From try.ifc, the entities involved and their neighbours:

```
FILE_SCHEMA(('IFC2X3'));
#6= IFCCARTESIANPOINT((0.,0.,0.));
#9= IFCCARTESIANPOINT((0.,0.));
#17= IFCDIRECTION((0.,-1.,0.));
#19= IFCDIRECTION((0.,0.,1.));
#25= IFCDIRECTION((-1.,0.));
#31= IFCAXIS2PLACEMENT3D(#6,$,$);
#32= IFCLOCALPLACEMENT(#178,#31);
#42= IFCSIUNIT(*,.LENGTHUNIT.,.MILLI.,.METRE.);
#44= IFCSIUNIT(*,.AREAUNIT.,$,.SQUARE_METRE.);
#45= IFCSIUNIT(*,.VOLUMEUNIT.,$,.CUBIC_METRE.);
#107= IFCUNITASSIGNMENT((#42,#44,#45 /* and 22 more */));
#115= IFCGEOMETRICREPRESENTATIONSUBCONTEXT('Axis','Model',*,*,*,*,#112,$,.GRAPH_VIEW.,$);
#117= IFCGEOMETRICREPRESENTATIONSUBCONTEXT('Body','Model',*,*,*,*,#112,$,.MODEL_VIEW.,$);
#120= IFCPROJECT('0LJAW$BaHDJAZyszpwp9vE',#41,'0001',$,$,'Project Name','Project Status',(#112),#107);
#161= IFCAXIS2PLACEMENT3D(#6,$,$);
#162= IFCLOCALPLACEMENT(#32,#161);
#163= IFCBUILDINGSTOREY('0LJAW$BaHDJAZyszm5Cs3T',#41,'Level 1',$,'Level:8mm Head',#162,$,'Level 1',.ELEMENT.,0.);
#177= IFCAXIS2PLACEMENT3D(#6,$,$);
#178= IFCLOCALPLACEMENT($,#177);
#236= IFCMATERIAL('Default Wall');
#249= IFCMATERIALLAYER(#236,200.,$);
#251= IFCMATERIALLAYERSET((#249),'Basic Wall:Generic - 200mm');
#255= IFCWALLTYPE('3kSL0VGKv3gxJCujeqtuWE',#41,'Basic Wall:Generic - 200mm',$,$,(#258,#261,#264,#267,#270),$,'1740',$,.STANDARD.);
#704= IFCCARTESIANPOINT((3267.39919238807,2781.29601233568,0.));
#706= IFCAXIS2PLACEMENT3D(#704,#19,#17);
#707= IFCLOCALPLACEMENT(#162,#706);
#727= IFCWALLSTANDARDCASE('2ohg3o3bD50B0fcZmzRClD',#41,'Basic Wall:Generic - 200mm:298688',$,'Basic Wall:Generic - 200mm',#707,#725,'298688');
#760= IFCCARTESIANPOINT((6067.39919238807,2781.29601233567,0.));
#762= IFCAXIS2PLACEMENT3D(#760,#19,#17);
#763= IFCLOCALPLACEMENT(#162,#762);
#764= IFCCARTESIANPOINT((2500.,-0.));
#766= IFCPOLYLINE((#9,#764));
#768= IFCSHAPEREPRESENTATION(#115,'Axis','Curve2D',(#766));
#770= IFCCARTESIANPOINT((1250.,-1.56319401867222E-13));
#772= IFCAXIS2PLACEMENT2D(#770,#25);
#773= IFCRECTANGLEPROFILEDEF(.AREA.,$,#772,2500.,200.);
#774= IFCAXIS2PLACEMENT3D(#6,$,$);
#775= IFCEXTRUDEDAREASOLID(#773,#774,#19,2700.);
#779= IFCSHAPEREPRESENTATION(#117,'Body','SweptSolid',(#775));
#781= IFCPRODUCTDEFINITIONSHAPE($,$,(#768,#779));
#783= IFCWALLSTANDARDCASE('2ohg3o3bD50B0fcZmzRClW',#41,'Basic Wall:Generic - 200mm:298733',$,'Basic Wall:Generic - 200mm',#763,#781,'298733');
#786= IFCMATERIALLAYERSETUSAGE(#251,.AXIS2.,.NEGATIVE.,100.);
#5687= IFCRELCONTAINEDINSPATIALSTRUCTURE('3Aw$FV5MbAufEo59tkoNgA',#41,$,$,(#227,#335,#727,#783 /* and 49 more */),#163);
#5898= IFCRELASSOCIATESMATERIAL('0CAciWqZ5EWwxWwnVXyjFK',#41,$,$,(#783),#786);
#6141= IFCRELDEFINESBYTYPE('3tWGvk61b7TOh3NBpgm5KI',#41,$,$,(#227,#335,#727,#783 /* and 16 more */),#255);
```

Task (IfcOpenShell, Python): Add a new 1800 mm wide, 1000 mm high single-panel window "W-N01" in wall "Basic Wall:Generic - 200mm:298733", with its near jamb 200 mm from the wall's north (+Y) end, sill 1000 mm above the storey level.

```python
import numpy as np
import ifcopenshell
import ifcopenshell.api.feature
import ifcopenshell.api.geometry
import ifcopenshell.api.root
import ifcopenshell.api.spatial
import ifcopenshell.api.type
import ifcopenshell.geom
import ifcopenshell.util.element
import ifcopenshell.util.placement
import ifcopenshell.util.representation
import ifcopenshell.util.shape
import ifcopenshell.util.unit

model = ifcopenshell.open("try.ifc")
unit_scale = ifcopenshell.util.unit.calculate_unit_scale(model)
settings = ifcopenshell.geom.settings()


def volume(element):
    """Net volume in cubic metres, openings subtracted."""
    shape = ifcopenshell.geom.create_shape(settings, element)
    return ifcopenshell.util.shape.get_volume(shape.geometry)


wall = model.by_id(783)
storey = ifcopenshell.util.element.get_container(wall, ifc_class="IfcBuildingStorey")
context = ifcopenshell.util.representation.get_context(model, "Model", "Body", "MODEL_VIEW")
before = volume(wall)

width, height, from_end, sill = 1.8, 1, 0.2, 1  # metres

# The wall runs along its own X axis, and the end named is its -X end.
wall_shape = ifcopenshell.geom.create_shape(settings, wall)
x, y, z = ifcopenshell.util.shape.get_vertices(wall_shape.geometry).T
start = x.min() + from_end
face, thickness = float(y.min()), float(y.max() - y.min())
wall_matrix = ifcopenshell.util.placement.get_local_placement(wall.ObjectPlacement)
level = ifcopenshell.util.placement.get_local_placement(storey.ObjectPlacement)[2, 3]


def in_wall(x, y):
    """Placement at x, y metres in the wall's axes, at sill height."""
    matrix = wall_matrix.copy()
    matrix[:, 3] = wall_matrix @ np.array([x / unit_scale, y / unit_scale, 0.0, 1.0])
    matrix[2, 3] = level + sill / unit_scale
    return matrix


# Opening: a box that overshoots both wall faces by 50 mm.
opening = ifcopenshell.api.root.create_entity(model, ifc_class="IfcOpeningElement")
box = ifcopenshell.api.geometry.add_wall_representation(
    model, context=context, length=width, height=height, thickness=thickness + 0.1
)
ifcopenshell.api.geometry.assign_representation(model, product=opening, representation=box)
ifcopenshell.api.geometry.edit_object_placement(model, product=opening, matrix=in_wall(start, face - 0.05), is_si=False)
ifcopenshell.api.feature.add_feature(model, feature=opening, element=wall)

window = ifcopenshell.api.root.create_entity(model, ifc_class="IfcWindow", name="W-N01")
window.OverallWidth, window.OverallHeight = width / unit_scale, height / unit_scale
body = ifcopenshell.api.geometry.add_window_representation(
    model,
    context=context,
    overall_width=window.OverallWidth,
    overall_height=window.OverallHeight,
    partition_type="SINGLE_PANEL",
)
ifcopenshell.api.geometry.assign_representation(model, product=window, representation=body)
ifcopenshell.api.spatial.assign_container(model, products=[window], relating_structure=storey)
fills = ifcopenshell.api.feature.add_filling(model, opening=opening, element=window)
fills.OwnerHistory = window.OwnerHistory  # required in IFC2X3

# IFC2X3 keeps the operation on the window style.
style = ifcopenshell.api.root.create_entity(model, ifc_class="IfcWindowStyle", name="W-N01")
style.OperationType, style.ConstructionType = "SINGLE_PANEL", "NOTDEFINED"
style.ParameterTakesPrecedence = style.Sizeable = False
ifcopenshell.api.type.assign_type(model, related_objects=[window], relating_type=style)

# Centre the window in the wall's thickness.
ifcopenshell.api.geometry.edit_object_placement(model, product=window, matrix=in_wall(start, face), is_si=False)
window_shape = ifcopenshell.geom.create_shape(settings, window)
depth = ifcopenshell.util.shape.get_vertices(window_shape.geometry)[:, 1]
offset = face + thickness / 2 - (depth.min() + depth.max()) / 2
ifcopenshell.api.geometry.edit_object_placement(model, product=window, matrix=in_wall(start, offset), is_si=False)

after = volume(wall)

print(f"wall volume {before:.3f} -> {after:.3f} m3")

model.write("try-out.ifc")
```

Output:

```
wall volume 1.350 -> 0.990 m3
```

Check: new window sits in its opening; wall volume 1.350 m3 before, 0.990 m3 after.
